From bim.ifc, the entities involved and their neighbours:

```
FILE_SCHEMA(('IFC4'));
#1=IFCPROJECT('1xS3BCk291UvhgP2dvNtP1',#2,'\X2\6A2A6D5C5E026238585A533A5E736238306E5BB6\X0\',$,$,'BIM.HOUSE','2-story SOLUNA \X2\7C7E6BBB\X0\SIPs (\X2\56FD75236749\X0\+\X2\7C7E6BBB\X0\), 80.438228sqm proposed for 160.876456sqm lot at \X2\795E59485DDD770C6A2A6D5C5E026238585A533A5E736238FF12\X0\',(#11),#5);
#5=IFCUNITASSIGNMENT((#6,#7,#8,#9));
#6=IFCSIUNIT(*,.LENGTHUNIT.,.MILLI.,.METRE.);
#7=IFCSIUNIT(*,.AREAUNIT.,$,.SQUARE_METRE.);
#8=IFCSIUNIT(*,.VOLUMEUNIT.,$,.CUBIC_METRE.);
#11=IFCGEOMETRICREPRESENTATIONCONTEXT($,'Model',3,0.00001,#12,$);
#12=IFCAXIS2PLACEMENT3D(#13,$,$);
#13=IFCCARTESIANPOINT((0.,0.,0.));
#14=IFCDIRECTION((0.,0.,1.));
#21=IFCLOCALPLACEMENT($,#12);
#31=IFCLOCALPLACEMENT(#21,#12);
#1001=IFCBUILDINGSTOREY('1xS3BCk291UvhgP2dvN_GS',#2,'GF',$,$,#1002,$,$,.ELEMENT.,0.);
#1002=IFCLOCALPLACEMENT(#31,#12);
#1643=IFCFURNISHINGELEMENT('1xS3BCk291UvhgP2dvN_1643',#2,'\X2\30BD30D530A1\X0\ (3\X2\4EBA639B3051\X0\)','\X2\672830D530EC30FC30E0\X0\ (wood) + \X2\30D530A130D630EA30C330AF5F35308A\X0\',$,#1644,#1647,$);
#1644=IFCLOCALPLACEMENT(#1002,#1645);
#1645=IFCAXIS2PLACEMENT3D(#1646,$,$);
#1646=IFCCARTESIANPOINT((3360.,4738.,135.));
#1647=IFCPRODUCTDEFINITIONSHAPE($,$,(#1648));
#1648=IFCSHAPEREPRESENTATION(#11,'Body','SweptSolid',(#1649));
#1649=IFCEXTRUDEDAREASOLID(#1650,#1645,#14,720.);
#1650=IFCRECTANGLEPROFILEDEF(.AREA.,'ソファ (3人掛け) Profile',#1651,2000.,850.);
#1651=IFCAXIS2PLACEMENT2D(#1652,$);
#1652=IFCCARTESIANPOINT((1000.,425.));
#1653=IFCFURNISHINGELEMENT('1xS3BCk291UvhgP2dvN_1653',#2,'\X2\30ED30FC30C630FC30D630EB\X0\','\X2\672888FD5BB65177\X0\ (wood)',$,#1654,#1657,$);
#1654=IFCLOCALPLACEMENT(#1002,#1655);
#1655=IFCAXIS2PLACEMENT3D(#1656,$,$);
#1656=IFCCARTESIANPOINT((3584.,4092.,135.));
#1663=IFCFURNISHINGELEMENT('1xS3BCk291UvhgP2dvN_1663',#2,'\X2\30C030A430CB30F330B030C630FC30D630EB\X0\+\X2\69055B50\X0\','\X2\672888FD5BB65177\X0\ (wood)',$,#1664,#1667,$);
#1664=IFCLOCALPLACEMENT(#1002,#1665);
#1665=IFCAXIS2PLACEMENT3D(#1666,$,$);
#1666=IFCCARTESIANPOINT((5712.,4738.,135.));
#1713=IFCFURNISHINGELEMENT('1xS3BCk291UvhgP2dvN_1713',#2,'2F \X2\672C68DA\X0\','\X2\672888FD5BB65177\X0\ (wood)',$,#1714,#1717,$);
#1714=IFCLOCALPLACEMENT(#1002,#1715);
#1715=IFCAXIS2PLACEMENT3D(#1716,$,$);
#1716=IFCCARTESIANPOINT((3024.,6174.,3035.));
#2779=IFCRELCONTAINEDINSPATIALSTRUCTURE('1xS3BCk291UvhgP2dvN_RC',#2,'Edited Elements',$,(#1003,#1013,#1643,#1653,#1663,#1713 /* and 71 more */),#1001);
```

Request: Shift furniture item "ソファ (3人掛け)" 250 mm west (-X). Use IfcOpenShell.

```python
import ifcopenshell
import ifcopenshell.api.geometry
import ifcopenshell.util.placement
import ifcopenshell.util.unit

model = ifcopenshell.open("bim.ifc")
unit_scale = ifcopenshell.util.unit.calculate_unit_scale(model)

item = model.by_guid("1xS3BCk291UvhgP2dvN_1643")
matrix = ifcopenshell.util.placement.get_local_placement(item.ObjectPlacement)
matrix[0, 3] -= 0.25 / unit_scale
ifcopenshell.api.geometry.edit_object_placement(model, product=item, matrix=matrix, is_si=False)

print(ifcopenshell.util.placement.get_local_placement(item.ObjectPlacement).round(3) + 0.0)

model.write("bim_updated.ifc")
```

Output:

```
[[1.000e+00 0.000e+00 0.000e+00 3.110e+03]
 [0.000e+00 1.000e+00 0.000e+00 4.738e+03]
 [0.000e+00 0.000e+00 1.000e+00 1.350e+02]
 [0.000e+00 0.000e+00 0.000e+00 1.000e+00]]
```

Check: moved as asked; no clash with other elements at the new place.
